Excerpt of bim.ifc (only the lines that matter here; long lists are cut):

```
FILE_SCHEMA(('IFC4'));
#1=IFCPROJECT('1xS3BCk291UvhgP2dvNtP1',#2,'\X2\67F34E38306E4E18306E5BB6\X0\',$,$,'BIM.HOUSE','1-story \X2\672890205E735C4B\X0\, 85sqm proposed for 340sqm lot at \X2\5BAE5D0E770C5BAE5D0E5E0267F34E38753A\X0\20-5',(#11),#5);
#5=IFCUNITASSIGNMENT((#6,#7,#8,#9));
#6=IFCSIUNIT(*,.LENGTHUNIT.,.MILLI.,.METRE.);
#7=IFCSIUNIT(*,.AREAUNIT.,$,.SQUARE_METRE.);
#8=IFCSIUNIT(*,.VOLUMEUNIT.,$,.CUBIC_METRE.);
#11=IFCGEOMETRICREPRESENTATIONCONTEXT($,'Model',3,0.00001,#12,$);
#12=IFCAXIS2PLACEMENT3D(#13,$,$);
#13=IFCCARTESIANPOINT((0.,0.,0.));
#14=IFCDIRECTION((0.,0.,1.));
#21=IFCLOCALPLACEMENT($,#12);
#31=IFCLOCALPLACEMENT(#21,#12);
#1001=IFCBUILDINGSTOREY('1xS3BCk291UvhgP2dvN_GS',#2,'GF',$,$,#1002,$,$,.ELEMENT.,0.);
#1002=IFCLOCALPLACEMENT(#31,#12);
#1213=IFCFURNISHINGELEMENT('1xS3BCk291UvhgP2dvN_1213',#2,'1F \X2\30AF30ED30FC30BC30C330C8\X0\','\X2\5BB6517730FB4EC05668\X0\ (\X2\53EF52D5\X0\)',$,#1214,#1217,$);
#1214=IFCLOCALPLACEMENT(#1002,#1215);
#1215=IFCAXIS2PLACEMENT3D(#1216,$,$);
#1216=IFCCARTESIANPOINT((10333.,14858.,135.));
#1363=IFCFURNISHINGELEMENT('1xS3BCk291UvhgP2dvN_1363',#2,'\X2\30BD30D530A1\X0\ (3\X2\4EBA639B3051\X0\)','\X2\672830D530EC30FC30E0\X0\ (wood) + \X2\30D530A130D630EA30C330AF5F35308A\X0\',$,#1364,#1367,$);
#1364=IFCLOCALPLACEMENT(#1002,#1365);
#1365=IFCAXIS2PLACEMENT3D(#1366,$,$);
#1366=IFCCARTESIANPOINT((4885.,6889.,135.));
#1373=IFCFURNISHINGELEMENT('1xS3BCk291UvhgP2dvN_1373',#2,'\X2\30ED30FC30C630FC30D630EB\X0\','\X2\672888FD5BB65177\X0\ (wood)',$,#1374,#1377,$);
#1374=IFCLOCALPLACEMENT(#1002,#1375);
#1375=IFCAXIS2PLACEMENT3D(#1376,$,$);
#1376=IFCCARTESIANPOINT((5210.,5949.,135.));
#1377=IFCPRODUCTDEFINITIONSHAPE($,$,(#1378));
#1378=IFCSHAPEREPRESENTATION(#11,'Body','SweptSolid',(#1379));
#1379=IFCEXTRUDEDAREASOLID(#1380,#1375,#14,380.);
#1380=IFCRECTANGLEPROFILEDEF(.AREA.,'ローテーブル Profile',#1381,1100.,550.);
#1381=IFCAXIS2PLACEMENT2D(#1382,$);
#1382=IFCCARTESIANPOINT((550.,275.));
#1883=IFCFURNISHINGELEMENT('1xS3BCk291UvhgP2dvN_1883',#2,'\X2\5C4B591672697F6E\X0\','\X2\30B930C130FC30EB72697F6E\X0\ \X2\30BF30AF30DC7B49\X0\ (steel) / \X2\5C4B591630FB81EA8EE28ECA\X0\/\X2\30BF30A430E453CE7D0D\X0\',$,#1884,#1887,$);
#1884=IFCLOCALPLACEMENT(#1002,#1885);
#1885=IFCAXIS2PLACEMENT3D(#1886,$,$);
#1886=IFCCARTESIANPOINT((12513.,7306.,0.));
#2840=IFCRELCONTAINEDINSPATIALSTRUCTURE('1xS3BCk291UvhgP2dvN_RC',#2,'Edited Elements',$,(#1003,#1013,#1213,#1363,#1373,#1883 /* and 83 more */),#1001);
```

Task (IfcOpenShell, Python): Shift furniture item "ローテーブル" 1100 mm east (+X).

```python
import ifcopenshell
import ifcopenshell.api.geometry
import ifcopenshell.util.placement
import ifcopenshell.util.unit

model = ifcopenshell.open("bim.ifc")
unit_scale = ifcopenshell.util.unit.calculate_unit_scale(model)

item = model.by_guid("1xS3BCk291UvhgP2dvN_1373")
matrix = ifcopenshell.util.placement.get_local_placement(item.ObjectPlacement)
matrix[0, 3] += 1.1 / unit_scale
ifcopenshell.api.geometry.edit_object_placement(model, product=item, matrix=matrix, is_si=False)

print(ifcopenshell.util.placement.get_local_placement(item.ObjectPlacement).round(3) + 0.0)

model.write("bim_v2.ifc")
```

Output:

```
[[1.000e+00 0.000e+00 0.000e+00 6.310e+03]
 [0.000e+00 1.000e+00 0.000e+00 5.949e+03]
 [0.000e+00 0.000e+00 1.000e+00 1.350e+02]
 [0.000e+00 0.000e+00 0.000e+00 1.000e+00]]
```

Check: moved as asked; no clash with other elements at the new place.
